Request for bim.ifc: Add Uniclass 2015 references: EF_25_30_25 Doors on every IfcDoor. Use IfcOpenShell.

First a look at what the model holds.

```python
import ifcopenshell

model = ifcopenshell.open("bim.ifc")
print(model.schema)
print("classifications:", [c.Name for c in model.by_type("IfcClassification")])
for ifc_class in ("IfcDoor", "IfcRoof", "IfcStair", "IfcWall", "IfcWindow"):
    print(ifc_class, len(model.by_type(ifc_class)))
```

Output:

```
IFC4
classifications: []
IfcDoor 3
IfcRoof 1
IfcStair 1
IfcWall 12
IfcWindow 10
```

```python
import ifcopenshell
import ifcopenshell.api.classification

model = ifcopenshell.open("bim.ifc")

system = ifcopenshell.api.classification.add_classification(model, classification="Uniclass 2015")

codes = {
    "IfcDoor": ("EF_25_30_25", "Doors"),
}
for ifc_class, (code, name) in codes.items():
    products = model.by_type(ifc_class)
    ifcopenshell.api.classification.add_reference(
        model, products=products, classification=system, identification=code, name=name
    )
    print(code, len(products))

model.write("bim_updated.ifc")
```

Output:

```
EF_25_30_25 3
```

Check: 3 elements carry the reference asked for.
